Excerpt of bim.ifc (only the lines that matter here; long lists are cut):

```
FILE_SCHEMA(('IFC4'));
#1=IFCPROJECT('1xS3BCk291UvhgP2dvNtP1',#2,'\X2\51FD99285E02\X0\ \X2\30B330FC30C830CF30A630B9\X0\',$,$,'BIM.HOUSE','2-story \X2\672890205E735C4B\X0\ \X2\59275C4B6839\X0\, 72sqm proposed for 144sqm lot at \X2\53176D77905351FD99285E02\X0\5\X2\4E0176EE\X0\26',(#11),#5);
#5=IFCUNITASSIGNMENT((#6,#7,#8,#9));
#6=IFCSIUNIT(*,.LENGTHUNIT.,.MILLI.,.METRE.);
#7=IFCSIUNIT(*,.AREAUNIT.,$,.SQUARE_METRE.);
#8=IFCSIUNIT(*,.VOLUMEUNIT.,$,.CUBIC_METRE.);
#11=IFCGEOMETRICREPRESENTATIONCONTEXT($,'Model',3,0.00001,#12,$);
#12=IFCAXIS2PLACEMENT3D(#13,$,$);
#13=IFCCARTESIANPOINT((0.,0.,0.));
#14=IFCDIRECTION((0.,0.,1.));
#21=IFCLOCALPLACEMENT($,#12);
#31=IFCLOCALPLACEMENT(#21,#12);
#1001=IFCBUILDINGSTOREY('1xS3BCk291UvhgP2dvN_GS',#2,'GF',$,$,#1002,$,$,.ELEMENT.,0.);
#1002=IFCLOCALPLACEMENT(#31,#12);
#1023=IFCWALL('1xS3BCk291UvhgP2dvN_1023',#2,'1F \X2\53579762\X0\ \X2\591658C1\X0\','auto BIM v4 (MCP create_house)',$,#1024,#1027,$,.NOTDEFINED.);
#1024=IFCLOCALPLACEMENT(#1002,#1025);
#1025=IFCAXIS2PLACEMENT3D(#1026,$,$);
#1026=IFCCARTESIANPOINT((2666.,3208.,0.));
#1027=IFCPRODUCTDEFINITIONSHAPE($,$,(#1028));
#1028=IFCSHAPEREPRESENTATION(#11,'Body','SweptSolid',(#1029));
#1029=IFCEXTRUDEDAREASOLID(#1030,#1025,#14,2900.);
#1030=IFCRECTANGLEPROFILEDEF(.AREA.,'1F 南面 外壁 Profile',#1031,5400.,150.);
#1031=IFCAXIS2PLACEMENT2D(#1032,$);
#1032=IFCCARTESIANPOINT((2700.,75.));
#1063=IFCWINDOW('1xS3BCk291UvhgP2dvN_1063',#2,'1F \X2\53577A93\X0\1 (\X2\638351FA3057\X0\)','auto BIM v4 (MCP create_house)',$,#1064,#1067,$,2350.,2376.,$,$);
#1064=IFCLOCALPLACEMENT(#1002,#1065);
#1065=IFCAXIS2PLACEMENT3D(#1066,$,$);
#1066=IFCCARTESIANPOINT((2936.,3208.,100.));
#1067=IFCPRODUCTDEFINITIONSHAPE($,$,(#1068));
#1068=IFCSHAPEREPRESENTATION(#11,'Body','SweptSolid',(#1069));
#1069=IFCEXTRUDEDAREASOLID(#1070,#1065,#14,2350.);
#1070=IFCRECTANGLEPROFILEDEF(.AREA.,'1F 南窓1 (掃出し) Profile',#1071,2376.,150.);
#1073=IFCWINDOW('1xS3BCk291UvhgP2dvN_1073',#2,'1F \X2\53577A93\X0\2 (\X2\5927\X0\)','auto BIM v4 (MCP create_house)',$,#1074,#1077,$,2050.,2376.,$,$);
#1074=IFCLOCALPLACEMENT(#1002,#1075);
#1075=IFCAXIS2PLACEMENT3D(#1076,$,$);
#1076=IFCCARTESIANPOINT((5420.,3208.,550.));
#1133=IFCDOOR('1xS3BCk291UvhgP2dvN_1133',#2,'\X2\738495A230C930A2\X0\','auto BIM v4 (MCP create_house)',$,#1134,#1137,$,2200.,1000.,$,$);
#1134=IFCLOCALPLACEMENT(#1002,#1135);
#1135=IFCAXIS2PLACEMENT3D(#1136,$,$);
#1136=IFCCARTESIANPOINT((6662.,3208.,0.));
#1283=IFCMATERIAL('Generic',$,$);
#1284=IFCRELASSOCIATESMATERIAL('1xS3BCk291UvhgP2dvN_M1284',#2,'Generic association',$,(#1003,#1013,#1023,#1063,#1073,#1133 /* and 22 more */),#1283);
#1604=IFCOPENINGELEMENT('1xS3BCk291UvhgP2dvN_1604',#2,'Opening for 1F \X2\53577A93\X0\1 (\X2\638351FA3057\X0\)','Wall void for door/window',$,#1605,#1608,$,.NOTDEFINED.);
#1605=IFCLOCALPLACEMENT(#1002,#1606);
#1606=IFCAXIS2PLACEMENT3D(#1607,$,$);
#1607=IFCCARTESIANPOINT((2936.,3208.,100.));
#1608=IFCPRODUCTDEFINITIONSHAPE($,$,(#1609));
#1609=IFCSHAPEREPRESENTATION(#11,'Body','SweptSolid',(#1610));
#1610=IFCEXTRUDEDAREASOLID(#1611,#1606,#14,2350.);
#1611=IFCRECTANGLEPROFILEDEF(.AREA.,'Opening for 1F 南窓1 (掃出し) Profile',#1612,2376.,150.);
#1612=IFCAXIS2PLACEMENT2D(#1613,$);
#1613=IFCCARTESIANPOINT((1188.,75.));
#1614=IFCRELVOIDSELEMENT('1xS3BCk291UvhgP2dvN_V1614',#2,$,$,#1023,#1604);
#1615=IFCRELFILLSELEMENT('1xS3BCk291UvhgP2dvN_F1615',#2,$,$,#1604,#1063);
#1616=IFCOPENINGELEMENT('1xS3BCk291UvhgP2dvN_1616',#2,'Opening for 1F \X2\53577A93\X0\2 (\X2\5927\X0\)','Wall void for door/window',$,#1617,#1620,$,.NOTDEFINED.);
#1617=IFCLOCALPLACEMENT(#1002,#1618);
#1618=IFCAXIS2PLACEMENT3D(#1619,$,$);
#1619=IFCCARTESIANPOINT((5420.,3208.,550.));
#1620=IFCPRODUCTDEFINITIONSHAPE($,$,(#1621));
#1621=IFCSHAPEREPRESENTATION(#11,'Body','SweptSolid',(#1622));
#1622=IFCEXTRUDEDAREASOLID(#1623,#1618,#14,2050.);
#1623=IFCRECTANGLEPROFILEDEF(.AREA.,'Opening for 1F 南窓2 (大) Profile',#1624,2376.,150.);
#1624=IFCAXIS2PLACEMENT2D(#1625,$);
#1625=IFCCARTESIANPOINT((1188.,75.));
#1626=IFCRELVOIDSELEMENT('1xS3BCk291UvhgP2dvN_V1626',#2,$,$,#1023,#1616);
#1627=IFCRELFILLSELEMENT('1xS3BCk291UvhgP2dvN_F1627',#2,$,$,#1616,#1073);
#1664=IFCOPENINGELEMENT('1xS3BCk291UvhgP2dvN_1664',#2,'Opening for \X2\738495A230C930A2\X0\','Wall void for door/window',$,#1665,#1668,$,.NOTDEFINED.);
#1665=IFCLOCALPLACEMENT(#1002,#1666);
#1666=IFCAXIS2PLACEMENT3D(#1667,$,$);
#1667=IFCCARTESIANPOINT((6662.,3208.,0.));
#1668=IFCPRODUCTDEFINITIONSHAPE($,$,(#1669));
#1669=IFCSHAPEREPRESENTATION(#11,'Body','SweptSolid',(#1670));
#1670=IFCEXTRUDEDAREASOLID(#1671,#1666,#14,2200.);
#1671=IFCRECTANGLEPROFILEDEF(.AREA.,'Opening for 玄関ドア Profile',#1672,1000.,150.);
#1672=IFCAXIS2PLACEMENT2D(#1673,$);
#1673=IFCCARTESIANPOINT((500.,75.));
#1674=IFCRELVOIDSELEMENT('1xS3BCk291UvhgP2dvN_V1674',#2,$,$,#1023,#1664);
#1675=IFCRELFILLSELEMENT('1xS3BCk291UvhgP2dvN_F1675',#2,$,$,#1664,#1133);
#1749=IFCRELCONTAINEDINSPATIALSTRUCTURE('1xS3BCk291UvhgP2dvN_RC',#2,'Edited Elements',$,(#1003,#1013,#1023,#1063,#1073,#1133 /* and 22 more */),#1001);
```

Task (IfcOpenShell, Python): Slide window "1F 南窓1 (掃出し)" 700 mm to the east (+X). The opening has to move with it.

```python
import ifcopenshell
import ifcopenshell.api.geometry
import ifcopenshell.util.placement
import ifcopenshell.util.unit

model = ifcopenshell.open("bim.ifc")
unit_scale = ifcopenshell.util.unit.calculate_unit_scale(model)

window = model.by_guid("1xS3BCk291UvhgP2dvN_1063")
opening = window.FillsVoids[0].RelatingOpeningElement
wall = opening.VoidsElements[0].RelatingBuildingElement

wall_matrix = ifcopenshell.util.placement.get_local_placement(wall.ObjectPlacement)
shift = wall_matrix[:3, 0] * 0.7 / unit_scale
before = ifcopenshell.util.placement.get_local_placement(window.ObjectPlacement)[:3, 3].copy()

# The window is not placed relative to its opening, so move both.
for product in (opening, window):
    matrix = ifcopenshell.util.placement.get_local_placement(product.ObjectPlacement)
    matrix[:3, 3] += shift
    ifcopenshell.api.geometry.edit_object_placement(model, product=product, matrix=matrix, is_si=False)

after = ifcopenshell.util.placement.get_local_placement(window.ObjectPlacement)[:3, 3]
print("window moved by", (after - before).round(3) + 0.0)

model.write("bim_edited.ifc")
```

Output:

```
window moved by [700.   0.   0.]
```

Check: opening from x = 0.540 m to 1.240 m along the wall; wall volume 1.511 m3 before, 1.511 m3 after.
